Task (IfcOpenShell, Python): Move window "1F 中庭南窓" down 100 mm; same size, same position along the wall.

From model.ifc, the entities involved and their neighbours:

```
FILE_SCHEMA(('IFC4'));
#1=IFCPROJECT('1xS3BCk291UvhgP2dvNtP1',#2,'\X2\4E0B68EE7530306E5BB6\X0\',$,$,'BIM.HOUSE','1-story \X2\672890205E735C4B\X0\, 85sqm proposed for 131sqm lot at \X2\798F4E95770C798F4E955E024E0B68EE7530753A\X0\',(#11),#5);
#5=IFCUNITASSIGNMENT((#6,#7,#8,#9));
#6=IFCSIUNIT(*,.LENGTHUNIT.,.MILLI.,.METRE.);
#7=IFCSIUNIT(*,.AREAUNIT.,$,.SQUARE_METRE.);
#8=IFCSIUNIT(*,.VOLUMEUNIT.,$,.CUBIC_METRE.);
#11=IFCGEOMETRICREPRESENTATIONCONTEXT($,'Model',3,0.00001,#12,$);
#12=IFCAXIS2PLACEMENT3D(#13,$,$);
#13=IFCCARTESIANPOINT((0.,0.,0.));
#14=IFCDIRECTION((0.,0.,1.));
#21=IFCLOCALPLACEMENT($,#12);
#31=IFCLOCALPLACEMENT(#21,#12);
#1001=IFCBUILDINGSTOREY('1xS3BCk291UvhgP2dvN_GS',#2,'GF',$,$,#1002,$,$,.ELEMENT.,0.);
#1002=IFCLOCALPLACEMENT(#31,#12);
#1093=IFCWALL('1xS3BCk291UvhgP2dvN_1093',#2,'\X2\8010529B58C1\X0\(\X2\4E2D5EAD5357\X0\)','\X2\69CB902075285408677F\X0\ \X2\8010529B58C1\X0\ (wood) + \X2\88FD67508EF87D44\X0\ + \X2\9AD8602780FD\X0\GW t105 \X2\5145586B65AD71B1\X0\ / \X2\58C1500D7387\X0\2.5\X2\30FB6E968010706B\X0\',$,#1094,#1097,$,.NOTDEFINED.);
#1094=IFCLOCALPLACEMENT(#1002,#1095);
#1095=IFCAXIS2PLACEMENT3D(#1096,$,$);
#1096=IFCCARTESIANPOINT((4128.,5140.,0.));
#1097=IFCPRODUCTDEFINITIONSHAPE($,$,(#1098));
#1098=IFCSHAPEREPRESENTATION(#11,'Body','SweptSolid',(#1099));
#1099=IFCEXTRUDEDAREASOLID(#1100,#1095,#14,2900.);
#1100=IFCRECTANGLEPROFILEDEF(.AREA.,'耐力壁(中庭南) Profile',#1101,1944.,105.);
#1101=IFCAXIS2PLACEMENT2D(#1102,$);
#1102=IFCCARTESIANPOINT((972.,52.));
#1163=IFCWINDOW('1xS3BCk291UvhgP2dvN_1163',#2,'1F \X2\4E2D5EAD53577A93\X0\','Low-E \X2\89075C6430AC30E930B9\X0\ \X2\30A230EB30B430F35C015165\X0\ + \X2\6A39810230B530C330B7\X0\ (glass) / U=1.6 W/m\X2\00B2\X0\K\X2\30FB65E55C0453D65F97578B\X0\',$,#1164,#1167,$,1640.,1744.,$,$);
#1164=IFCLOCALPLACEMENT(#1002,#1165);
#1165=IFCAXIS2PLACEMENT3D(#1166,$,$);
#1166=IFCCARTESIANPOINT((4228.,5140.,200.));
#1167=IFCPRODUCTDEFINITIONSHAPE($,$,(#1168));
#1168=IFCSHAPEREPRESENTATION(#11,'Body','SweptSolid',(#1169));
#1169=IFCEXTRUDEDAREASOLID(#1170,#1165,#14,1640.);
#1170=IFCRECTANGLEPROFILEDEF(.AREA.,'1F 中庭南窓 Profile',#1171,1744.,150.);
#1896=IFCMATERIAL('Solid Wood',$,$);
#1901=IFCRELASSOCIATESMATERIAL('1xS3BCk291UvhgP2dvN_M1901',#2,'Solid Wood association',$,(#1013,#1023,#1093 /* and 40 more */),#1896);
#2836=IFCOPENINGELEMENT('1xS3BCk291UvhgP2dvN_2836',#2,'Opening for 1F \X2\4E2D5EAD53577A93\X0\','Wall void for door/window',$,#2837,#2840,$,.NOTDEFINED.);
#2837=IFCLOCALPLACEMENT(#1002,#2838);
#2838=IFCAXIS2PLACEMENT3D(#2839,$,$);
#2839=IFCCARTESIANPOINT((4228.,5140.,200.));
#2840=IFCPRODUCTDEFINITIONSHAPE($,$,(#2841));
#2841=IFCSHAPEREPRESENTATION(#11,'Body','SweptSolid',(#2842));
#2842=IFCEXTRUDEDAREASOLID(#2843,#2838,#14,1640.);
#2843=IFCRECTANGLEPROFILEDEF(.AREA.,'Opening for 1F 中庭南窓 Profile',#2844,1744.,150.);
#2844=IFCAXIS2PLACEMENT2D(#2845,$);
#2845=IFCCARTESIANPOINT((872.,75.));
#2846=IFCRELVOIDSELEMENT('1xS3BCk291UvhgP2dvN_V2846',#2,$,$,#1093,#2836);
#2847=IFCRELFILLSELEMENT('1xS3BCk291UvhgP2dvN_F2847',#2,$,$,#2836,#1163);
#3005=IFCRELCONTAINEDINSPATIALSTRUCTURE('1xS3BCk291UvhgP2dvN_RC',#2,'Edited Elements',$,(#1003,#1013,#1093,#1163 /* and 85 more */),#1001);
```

```python
import numpy as np
import ifcopenshell
import ifcopenshell.api.geometry
import ifcopenshell.util.placement
import ifcopenshell.util.unit

model = ifcopenshell.open("model.ifc")
unit_scale = ifcopenshell.util.unit.calculate_unit_scale(model)

window = model.by_id(1163)
opening = window.FillsVoids[0].RelatingOpeningElement
dz = -0.1 / unit_scale

shift = np.array([0.0, 0.0, dz])
# The window is not placed relative to its opening, so move both.
for product in (opening, window):
    matrix = ifcopenshell.util.placement.get_local_placement(product.ObjectPlacement)
    matrix[:3, 3] += shift
    ifcopenshell.api.geometry.edit_object_placement(model, product=product, matrix=matrix, is_si=False)

print(f"moved by {dz * unit_scale:+.3f} m")

model.write("model_updated.ifc")
```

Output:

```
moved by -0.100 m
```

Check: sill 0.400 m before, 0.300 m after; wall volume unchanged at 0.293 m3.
